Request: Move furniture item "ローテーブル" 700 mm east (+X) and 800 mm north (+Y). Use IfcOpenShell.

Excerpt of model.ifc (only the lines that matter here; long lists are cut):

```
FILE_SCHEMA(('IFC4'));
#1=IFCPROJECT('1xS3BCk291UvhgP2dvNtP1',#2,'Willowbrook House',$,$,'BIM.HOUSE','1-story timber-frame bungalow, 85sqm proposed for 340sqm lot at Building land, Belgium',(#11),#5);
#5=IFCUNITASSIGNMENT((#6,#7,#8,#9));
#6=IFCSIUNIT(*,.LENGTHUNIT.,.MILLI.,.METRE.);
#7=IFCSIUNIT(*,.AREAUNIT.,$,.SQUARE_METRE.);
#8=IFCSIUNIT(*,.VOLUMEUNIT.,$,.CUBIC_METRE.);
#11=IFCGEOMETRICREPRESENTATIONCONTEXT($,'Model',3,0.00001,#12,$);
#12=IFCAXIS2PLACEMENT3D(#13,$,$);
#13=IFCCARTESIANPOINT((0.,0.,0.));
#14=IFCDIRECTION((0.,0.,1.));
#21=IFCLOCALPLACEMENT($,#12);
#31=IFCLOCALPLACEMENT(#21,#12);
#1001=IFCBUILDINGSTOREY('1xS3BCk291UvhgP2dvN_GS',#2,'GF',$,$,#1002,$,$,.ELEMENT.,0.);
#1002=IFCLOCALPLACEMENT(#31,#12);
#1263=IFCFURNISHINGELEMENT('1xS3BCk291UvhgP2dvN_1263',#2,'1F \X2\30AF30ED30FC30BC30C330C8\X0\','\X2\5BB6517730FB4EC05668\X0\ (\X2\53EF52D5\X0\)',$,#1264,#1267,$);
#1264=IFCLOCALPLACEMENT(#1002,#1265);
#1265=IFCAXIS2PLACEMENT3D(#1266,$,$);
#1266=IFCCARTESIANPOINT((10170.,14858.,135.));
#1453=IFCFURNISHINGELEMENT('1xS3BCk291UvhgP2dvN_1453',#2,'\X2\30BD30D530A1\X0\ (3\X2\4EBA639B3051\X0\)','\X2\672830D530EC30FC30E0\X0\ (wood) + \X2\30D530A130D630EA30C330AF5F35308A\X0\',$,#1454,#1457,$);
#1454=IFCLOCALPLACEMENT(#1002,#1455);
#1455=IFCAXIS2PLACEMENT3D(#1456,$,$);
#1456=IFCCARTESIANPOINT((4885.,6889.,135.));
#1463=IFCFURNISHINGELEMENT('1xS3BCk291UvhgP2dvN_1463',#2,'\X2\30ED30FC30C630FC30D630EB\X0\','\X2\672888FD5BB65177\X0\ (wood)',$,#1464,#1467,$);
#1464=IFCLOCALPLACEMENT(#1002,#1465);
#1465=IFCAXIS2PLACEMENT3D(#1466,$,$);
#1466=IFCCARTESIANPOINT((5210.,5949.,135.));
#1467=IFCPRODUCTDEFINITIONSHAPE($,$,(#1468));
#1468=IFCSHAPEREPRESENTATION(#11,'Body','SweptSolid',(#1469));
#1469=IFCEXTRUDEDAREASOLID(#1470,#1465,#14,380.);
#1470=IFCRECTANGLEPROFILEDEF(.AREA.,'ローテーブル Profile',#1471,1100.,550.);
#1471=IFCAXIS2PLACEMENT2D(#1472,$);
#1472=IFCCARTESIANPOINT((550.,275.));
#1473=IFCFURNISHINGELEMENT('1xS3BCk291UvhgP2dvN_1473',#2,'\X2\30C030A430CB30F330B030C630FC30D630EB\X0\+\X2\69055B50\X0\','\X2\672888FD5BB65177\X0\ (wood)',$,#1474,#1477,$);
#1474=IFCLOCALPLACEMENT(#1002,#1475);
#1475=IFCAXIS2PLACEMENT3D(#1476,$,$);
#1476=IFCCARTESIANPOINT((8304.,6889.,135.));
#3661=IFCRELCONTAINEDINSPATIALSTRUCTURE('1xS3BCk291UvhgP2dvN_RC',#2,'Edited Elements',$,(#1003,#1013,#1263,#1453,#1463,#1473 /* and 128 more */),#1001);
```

```python
import ifcopenshell
import ifcopenshell.api.geometry
import ifcopenshell.util.placement
import ifcopenshell.util.unit

model = ifcopenshell.open("model.ifc")
unit_scale = ifcopenshell.util.unit.calculate_unit_scale(model)

item = model.by_guid("1xS3BCk291UvhgP2dvN_1463")
matrix = ifcopenshell.util.placement.get_local_placement(item.ObjectPlacement)
matrix[0, 3] += 0.7 / unit_scale
matrix[1, 3] += 0.8 / unit_scale
ifcopenshell.api.geometry.edit_object_placement(model, product=item, matrix=matrix, is_si=False)

print(ifcopenshell.util.placement.get_local_placement(item.ObjectPlacement).round(3) + 0.0)

model.write("model_rev.ifc")
```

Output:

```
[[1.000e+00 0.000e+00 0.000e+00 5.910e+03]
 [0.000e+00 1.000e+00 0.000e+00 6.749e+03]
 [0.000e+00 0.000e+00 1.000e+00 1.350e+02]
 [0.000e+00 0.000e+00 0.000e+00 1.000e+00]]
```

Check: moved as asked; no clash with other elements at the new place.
